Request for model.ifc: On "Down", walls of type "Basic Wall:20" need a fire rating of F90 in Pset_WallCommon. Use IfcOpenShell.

First a look at what the model holds.

```python
import ifcopenshell
import ifcopenshell.util.element

model = ifcopenshell.open("model.ifc")
print(model.schema)
storey = next(s for s in model.by_type("IfcBuildingStorey") if s.Name == "Down")
walls = [e for e in ifcopenshell.util.element.get_decomposition(storey) if e.is_a("IfcWall")]
seen = {}
for e in walls:
    element_type = ifcopenshell.util.element.get_type(e)
    key = (element_type.Name if element_type != e and element_type else None, ifcopenshell.util.element.get_pset(e, "Pset_WallCommon", "FireRating"))
    seen[key] = seen.get(key, 0) + 1
for (name, value), count in sorted(seen.items(), key=str):
    print(count, "x", name, "|", value)
```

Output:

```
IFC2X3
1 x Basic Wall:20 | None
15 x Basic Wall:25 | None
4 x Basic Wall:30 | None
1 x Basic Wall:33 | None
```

```python
import ifcopenshell
import ifcopenshell.api.pset
import ifcopenshell.util.element

model = ifcopenshell.open("model.ifc")

storey = next(s for s in model.by_type("IfcBuildingStorey") if s.Name == "Down")
walls = [e for e in ifcopenshell.util.element.get_decomposition(storey) if e.is_a("IfcWall")]

count = 0
for e in walls:
    element_type = ifcopenshell.util.element.get_type(e)
    if element_type in (None, e) or element_type.Name != "Basic Wall:20":
        continue
    # add_pset returns the element's existing set when there is one.
    pset = ifcopenshell.api.pset.add_pset(model, product=e, name="Pset_WallCommon")
    ifcopenshell.api.pset.edit_pset(model, pset=pset, properties={"FireRating": "F90"})
    count += 1

print(count, "walls updated")

model.write("model_updated.ifc")
```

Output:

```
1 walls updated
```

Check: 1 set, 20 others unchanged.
